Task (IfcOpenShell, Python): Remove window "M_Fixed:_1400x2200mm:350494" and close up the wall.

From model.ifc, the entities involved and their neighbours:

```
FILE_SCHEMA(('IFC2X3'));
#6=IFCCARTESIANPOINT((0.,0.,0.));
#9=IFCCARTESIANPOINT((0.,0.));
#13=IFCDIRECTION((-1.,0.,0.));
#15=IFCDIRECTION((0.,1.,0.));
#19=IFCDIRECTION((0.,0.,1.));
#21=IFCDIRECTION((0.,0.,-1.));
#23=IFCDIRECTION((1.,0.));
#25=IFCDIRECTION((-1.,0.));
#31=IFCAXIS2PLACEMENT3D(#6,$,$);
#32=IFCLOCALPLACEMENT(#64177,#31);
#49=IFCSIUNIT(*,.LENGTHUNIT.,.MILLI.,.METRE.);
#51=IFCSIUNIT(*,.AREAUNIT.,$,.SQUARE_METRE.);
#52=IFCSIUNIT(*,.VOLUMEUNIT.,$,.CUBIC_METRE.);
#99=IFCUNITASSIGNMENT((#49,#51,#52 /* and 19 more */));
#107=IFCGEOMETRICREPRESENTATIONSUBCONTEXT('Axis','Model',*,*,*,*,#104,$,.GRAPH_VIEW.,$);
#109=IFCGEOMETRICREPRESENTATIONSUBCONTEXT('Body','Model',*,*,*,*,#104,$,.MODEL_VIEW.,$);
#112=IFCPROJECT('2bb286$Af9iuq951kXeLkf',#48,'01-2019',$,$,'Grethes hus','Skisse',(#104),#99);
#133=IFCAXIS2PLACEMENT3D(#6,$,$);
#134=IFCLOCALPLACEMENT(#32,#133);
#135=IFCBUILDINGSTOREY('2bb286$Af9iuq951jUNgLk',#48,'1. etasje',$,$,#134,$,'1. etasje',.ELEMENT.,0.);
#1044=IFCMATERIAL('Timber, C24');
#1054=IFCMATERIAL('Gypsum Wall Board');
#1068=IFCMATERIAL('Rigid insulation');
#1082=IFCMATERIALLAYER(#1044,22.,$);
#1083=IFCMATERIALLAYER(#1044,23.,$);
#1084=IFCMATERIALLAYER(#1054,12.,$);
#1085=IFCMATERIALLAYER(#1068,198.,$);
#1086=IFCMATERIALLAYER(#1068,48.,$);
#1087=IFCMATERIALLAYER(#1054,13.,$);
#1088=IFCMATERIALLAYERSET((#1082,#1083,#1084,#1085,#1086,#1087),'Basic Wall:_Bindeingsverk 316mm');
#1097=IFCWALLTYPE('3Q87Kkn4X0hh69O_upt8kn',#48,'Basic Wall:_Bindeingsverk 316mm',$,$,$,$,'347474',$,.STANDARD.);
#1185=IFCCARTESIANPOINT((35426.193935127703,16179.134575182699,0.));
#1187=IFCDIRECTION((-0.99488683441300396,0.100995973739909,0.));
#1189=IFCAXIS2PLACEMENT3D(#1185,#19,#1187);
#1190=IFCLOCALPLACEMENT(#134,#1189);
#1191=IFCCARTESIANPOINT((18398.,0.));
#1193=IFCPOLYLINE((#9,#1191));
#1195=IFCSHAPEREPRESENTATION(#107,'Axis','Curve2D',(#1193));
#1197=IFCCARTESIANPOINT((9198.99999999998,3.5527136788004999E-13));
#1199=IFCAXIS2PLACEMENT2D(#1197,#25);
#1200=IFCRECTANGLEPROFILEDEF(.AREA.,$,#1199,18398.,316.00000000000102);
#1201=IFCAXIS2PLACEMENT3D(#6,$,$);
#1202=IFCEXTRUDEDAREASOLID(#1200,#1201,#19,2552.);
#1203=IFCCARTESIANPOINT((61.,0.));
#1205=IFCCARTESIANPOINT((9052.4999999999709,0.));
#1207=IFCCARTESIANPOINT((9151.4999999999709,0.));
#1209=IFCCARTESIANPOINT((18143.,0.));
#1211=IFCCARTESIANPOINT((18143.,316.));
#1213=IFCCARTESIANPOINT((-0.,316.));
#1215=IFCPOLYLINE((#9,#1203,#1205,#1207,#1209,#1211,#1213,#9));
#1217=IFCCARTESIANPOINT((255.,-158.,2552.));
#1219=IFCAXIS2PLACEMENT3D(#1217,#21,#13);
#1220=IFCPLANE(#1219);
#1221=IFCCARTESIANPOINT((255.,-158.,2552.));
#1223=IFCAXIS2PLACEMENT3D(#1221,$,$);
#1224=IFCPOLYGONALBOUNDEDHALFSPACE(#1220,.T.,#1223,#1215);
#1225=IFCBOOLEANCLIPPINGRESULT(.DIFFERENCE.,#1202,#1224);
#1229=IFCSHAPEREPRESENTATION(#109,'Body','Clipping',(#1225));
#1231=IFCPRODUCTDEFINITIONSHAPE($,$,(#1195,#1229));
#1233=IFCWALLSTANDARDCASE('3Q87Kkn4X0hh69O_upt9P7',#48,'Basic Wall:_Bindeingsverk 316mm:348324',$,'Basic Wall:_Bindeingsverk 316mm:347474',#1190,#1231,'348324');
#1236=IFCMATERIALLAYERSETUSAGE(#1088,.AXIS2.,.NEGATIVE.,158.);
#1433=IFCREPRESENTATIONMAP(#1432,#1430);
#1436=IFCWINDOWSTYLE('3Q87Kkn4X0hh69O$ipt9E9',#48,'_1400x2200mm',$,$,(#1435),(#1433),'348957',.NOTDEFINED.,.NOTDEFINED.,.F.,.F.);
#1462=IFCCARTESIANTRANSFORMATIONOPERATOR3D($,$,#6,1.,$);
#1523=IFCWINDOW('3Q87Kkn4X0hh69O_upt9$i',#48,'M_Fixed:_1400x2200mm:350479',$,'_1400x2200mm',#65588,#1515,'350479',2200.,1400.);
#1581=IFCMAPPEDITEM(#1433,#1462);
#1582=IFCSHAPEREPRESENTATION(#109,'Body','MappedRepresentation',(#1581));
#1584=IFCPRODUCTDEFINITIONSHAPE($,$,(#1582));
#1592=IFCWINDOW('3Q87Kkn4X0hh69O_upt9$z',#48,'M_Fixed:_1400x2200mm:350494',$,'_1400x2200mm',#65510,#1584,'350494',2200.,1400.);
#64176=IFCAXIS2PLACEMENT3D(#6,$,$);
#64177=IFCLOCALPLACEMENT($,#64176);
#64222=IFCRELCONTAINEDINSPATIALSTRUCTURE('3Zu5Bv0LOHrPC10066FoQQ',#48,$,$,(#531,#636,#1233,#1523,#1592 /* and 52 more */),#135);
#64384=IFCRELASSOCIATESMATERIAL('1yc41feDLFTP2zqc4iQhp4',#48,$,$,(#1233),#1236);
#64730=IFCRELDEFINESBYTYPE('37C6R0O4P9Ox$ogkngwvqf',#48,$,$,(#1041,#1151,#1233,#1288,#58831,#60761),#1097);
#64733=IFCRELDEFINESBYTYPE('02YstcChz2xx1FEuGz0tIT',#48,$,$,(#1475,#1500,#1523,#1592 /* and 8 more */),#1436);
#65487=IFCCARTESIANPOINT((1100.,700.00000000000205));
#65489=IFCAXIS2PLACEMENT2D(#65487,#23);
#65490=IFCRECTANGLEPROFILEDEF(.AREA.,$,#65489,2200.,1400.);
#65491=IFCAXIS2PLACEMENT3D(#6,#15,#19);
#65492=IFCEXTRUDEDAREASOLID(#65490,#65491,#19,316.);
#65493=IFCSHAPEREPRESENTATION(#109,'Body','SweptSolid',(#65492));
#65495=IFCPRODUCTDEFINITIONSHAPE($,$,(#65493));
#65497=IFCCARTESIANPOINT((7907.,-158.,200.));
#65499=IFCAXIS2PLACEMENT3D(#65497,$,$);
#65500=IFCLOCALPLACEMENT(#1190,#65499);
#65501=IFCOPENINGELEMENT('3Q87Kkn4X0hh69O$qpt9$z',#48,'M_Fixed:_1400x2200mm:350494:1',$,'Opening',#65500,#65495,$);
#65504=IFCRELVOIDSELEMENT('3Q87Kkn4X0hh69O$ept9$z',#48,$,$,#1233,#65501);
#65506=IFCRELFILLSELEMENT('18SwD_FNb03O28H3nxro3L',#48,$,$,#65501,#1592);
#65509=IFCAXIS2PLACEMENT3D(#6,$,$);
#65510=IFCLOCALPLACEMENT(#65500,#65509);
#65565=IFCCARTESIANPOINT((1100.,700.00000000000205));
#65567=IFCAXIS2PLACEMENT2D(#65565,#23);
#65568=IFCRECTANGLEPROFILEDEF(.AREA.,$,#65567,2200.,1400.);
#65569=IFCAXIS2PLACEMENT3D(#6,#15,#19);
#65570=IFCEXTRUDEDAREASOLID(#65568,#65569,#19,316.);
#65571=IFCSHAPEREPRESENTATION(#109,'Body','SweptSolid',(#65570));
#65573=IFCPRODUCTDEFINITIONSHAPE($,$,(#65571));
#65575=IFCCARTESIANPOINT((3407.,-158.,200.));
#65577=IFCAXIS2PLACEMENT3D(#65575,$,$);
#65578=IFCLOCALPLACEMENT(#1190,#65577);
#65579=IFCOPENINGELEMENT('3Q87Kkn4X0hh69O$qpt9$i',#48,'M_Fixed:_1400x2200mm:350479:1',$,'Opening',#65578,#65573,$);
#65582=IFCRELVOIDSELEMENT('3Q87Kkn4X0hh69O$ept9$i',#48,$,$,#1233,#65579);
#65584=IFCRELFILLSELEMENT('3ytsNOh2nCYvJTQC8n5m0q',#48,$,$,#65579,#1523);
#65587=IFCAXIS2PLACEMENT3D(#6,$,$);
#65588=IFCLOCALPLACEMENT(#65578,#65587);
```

```python
import ifcopenshell
import ifcopenshell.api.feature
import ifcopenshell.api.root
import ifcopenshell.geom
import ifcopenshell.util.shape

model = ifcopenshell.open("model.ifc")
settings = ifcopenshell.geom.settings()


def volume(element):
    """Net volume in cubic metres, openings subtracted."""
    shape = ifcopenshell.geom.create_shape(settings, element)
    return ifcopenshell.util.shape.get_volume(shape.geometry)


window = model.by_guid("3Q87Kkn4X0hh69O_upt9$z")
opening = window.FillsVoids[0].RelatingOpeningElement
wall = opening.VoidsElements[0].RelatingBuildingElement
before = volume(wall)

ifcopenshell.api.root.remove_product(model, product=window)
ifcopenshell.api.feature.remove_feature(model, feature=opening)

after = volume(wall)

print(f"wall volume {before:.3f} -> {after:.3f} m3")

model.write("model_rev.ifc")
```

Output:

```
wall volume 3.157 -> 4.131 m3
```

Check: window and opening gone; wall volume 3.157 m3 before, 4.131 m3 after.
